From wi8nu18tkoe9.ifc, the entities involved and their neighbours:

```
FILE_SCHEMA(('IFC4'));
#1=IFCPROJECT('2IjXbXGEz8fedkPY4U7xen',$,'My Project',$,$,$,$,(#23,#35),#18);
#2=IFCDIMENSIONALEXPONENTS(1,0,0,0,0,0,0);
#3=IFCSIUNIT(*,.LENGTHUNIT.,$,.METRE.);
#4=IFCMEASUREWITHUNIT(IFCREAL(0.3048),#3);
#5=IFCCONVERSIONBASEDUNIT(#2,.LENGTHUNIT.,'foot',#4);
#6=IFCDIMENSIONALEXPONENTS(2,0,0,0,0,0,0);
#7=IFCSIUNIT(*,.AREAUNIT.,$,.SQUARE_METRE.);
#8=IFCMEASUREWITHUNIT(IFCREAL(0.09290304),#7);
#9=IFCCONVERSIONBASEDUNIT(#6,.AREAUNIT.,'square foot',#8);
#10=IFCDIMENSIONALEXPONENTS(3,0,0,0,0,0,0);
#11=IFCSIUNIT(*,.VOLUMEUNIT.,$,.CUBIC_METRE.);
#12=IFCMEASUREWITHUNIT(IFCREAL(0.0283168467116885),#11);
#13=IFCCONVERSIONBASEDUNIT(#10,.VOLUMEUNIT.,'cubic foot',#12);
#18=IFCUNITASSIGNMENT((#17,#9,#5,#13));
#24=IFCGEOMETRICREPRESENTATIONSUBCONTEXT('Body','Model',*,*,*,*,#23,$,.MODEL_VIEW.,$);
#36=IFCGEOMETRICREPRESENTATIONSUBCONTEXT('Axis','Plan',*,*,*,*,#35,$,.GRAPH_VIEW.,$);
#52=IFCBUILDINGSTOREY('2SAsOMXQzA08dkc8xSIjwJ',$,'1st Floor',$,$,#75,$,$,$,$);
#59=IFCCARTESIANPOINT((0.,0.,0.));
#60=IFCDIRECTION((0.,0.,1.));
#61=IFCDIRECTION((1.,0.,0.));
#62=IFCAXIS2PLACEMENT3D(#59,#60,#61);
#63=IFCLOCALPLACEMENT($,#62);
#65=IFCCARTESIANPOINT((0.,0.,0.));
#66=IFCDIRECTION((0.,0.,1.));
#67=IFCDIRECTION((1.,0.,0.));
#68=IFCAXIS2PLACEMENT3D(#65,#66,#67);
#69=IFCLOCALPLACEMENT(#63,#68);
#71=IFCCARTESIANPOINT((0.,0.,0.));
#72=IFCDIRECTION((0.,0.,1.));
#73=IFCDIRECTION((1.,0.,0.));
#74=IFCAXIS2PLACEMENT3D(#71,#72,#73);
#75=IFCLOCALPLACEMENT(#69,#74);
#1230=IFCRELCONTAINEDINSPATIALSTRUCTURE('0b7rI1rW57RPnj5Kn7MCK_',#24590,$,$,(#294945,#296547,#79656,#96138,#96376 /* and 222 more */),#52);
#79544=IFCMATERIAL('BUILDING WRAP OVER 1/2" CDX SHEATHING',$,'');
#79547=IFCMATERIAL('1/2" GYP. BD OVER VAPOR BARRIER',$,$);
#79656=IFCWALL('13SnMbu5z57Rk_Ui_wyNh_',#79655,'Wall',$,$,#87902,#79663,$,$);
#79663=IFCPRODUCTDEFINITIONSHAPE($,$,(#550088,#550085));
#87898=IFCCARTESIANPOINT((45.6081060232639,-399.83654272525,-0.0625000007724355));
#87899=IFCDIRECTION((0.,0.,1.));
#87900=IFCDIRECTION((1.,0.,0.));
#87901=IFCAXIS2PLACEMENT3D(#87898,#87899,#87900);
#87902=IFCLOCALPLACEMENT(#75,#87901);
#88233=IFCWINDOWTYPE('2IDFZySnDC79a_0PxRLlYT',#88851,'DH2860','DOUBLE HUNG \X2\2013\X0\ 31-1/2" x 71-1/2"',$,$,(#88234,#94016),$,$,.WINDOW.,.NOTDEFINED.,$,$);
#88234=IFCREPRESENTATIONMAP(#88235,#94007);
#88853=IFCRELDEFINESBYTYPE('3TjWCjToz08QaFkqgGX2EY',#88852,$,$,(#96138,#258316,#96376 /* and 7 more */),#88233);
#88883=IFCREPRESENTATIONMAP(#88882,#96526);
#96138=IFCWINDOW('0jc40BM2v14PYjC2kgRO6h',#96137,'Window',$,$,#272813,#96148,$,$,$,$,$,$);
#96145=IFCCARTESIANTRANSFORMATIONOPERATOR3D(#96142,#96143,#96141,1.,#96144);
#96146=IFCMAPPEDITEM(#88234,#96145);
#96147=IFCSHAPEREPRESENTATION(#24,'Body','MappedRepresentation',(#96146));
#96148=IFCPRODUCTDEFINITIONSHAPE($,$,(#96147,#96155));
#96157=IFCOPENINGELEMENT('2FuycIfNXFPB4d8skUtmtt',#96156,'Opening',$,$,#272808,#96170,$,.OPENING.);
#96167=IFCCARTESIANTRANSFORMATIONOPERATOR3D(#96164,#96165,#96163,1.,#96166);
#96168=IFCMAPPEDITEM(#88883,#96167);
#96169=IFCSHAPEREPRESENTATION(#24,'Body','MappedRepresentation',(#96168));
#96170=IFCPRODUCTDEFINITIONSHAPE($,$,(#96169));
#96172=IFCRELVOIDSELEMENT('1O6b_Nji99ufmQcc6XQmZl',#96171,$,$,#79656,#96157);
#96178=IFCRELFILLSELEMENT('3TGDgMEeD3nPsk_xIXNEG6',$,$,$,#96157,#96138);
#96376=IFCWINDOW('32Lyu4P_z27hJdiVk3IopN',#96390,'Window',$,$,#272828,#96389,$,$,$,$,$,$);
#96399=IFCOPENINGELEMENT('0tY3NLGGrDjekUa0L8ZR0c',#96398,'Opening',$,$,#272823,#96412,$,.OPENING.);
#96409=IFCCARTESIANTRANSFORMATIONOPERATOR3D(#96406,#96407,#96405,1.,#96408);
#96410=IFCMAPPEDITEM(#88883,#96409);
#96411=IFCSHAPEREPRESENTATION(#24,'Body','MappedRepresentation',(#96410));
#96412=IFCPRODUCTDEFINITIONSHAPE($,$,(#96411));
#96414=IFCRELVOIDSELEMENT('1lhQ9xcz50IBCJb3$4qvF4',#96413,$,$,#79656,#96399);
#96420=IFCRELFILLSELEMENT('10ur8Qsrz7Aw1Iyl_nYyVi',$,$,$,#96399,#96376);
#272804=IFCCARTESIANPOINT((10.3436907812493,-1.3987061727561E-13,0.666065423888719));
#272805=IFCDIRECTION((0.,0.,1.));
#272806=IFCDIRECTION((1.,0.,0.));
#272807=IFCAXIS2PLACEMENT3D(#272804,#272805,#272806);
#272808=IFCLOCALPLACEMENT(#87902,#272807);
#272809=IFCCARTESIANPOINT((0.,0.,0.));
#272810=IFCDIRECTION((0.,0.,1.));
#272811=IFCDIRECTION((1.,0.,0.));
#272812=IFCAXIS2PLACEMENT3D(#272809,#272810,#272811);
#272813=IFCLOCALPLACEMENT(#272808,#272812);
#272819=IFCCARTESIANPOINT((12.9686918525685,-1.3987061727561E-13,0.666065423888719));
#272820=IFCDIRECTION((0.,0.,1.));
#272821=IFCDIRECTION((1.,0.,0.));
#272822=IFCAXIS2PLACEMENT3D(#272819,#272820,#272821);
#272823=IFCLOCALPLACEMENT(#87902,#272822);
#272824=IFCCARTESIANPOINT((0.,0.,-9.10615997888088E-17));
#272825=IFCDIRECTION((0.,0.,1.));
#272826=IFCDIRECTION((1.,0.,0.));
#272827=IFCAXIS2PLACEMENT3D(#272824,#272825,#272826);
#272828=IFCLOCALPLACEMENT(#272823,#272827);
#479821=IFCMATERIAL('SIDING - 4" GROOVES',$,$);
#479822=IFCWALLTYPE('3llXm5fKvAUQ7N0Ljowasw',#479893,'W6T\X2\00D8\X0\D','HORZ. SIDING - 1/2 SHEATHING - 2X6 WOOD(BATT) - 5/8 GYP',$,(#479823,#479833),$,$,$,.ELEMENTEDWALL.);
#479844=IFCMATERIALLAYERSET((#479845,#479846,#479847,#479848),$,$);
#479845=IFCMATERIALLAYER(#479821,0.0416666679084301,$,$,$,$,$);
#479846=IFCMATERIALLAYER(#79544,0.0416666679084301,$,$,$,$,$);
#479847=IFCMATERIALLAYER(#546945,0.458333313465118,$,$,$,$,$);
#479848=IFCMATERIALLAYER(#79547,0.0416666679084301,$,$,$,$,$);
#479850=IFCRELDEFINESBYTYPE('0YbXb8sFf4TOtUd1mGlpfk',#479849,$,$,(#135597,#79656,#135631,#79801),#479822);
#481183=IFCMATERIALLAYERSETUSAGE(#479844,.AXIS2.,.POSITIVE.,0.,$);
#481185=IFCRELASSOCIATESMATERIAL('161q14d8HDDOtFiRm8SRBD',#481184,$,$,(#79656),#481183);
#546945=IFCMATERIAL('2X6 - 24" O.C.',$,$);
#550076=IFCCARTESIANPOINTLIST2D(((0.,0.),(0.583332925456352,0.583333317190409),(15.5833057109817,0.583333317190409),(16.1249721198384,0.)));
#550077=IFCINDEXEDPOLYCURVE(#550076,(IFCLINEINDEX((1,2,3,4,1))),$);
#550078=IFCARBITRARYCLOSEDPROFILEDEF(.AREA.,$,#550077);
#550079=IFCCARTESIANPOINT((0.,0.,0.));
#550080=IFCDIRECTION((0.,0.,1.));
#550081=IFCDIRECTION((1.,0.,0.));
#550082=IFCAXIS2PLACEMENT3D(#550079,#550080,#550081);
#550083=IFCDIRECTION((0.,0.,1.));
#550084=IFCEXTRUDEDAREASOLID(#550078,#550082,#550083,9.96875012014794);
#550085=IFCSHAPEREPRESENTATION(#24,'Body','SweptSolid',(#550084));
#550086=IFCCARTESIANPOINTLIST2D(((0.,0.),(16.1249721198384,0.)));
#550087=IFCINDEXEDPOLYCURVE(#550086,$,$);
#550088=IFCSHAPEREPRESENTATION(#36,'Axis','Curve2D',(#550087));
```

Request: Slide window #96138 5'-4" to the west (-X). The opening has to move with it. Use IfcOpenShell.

```python
import ifcopenshell
import ifcopenshell.api.geometry
import ifcopenshell.util.placement
import ifcopenshell.util.unit

model = ifcopenshell.open("wi8nu18tkoe9.ifc")
unit_scale = ifcopenshell.util.unit.calculate_unit_scale(model)

window = model.by_guid("0jc40BM2v14PYjC2kgRO6h")
opening = window.FillsVoids[0].RelatingOpeningElement
wall = opening.VoidsElements[0].RelatingBuildingElement

wall_matrix = ifcopenshell.util.placement.get_local_placement(wall.ObjectPlacement)
shift = wall_matrix[:3, 0] * -64 * 0.0254 / unit_scale
before = ifcopenshell.util.placement.get_local_placement(window.ObjectPlacement)[:3, 3].copy()

# The window is placed relative to its opening, so it follows when the opening moves.
matrix = ifcopenshell.util.placement.get_local_placement(opening.ObjectPlacement)
matrix[:3, 3] += shift
ifcopenshell.api.geometry.edit_object_placement(
    model, product=opening, matrix=matrix, is_si=False, should_transform_children=True
)

after = ifcopenshell.util.placement.get_local_placement(window.ObjectPlacement)[:3, 3]
print("window moved by", (after - before).round(3) + 0.0)

model.write("wi8nu18tkoe9-out.ifc")
```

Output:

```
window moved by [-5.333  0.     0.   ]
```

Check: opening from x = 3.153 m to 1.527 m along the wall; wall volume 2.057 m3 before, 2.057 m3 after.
